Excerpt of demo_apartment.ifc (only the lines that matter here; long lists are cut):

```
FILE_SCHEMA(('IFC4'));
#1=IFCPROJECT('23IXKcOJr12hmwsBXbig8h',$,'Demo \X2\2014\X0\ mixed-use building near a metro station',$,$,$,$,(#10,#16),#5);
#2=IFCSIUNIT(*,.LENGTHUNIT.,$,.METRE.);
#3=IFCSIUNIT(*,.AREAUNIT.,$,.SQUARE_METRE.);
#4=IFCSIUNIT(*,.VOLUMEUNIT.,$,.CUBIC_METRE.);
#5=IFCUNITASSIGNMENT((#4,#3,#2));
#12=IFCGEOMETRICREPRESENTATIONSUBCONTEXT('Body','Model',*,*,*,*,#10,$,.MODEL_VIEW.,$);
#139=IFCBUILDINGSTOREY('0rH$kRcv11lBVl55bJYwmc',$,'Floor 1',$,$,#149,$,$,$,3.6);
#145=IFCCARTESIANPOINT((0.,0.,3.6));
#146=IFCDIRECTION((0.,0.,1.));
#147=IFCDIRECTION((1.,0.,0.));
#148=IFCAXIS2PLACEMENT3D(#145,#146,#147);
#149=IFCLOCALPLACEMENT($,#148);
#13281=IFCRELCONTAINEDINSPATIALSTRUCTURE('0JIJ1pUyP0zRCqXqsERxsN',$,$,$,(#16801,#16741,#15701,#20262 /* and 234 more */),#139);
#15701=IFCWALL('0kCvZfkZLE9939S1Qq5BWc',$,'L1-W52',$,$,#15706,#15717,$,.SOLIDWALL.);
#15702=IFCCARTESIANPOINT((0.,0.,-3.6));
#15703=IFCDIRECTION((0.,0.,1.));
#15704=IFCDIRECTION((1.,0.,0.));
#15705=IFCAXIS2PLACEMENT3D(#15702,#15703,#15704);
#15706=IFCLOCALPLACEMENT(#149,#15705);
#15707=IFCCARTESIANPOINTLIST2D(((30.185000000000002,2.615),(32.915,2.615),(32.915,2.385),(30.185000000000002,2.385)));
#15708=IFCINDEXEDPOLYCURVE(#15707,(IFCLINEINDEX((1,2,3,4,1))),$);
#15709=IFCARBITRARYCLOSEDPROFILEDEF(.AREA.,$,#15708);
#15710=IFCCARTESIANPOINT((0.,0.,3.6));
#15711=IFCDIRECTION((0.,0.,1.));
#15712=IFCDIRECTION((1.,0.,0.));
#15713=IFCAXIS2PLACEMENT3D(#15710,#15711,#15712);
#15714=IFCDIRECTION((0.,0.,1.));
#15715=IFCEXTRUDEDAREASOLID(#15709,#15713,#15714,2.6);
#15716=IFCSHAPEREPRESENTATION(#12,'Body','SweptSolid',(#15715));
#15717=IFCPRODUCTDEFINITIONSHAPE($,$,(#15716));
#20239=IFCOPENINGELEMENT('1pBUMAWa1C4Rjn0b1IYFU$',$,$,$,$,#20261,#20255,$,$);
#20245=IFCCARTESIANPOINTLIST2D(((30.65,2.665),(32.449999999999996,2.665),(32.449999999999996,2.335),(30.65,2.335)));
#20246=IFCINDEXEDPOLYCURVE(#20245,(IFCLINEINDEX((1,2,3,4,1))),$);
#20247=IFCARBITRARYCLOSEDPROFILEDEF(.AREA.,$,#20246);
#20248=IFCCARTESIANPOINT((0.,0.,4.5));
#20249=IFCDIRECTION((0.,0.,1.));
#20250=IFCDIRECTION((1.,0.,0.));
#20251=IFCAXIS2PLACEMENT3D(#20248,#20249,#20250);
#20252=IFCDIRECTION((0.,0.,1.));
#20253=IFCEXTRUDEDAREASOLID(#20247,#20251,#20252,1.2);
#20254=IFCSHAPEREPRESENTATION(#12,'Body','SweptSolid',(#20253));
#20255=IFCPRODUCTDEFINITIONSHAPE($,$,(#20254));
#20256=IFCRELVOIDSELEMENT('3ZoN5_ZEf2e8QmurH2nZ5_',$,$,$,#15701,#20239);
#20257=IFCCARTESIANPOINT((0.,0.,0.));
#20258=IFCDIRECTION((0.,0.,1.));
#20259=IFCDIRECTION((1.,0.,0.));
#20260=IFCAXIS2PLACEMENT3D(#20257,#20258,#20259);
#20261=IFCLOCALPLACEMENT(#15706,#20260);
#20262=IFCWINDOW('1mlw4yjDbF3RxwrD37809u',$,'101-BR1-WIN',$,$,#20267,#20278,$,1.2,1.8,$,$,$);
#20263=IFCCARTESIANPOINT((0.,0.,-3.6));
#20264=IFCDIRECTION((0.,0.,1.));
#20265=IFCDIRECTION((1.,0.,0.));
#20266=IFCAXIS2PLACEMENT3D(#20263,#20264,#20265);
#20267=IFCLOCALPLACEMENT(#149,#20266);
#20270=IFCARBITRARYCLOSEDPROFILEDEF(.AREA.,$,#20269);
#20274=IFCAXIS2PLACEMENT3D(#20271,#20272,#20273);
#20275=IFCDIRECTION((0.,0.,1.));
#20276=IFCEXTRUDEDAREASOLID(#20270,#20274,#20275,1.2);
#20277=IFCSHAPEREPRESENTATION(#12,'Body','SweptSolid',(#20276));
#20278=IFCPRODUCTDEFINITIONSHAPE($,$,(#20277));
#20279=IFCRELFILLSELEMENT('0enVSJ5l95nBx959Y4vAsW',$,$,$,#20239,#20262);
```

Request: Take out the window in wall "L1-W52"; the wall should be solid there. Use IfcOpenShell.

```python
import ifcopenshell
import ifcopenshell.api.feature
import ifcopenshell.api.root
import ifcopenshell.geom
import ifcopenshell.util.shape

model = ifcopenshell.open("demo_apartment.ifc")
settings = ifcopenshell.geom.settings()


def volume(element):
    """Net volume in cubic metres, openings subtracted."""
    shape = ifcopenshell.geom.create_shape(settings, element)
    return ifcopenshell.util.shape.get_volume(shape.geometry)


window = model.by_guid("1mlw4yjDbF3RxwrD37809u")
opening = window.FillsVoids[0].RelatingOpeningElement
wall = opening.VoidsElements[0].RelatingBuildingElement
before = volume(wall)

ifcopenshell.api.root.remove_product(model, product=window)
ifcopenshell.api.feature.remove_feature(model, feature=opening)

after = volume(wall)

print(f"wall volume {before:.3f} -> {after:.3f} m3")

model.write("demo_apartment-out.ifc")
```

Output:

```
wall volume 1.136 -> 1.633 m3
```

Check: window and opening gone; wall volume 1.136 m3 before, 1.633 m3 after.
